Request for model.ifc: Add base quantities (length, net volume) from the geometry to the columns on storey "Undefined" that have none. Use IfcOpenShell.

First a look at what the model holds.

```python
import ifcopenshell
import ifcopenshell.util.element
import ifcopenshell.util.unit

model = ifcopenshell.open("model.ifc")
print(model.schema)
for unit_type in ("LENGTHUNIT", "AREAUNIT", "VOLUMEUNIT"):
    print(unit_type, ifcopenshell.util.unit.calculate_unit_scale(model, unit_type))
storey = next(s for s in model.by_type("IfcBuildingStorey") if s.Name == "Undefined")
columns = [e for e in ifcopenshell.util.element.get_decomposition(storey) if e.is_a("IfcColumn")]
for e in sorted(columns, key=lambda e: e.id()):
    print(e.id(), e.is_a(), e.Name, list(ifcopenshell.util.element.get_psets(e, qtos_only=True)), sep=" | ")
```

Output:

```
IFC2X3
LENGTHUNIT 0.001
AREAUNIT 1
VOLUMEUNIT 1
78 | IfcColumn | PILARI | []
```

```python
import ifcopenshell
import ifcopenshell.api.pset
import ifcopenshell.geom
import ifcopenshell.util.element
import ifcopenshell.util.shape
import ifcopenshell.util.unit

model = ifcopenshell.open("model.ifc")
unit_scale = ifcopenshell.util.unit.calculate_unit_scale(model)
volume_scale = ifcopenshell.util.unit.calculate_unit_scale(model, "VOLUMEUNIT")
settings = ifcopenshell.geom.settings()

storey = next(s for s in model.by_type("IfcBuildingStorey") if s.Name == "Undefined")
columns = [e for e in ifcopenshell.util.element.get_decomposition(storey) if e.is_a("IfcColumn")]

for e in sorted(columns, key=lambda e: e.id()):
    if ifcopenshell.util.element.get_psets(e, qtos_only=True, should_inherit=False):
        continue
    # Geometry comes back in metres, in the element's own axes.
    shape = ifcopenshell.geom.create_shape(settings, e)
    values = {
        "Length": ifcopenshell.util.shape.get_z(shape.geometry) / unit_scale,
        "NetVolume": ifcopenshell.util.shape.get_volume(shape.geometry) / volume_scale,
    }
    qto = ifcopenshell.api.pset.add_qto(model, product=e, name="BaseQuantities")
    ifcopenshell.api.pset.edit_qto(model, qto=qto, properties=values)
    print(e.id(), {k: round(v, 3) for k, v in values.items()})

model.write("model-out.ifc")
```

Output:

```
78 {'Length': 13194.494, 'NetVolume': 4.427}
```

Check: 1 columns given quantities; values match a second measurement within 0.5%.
